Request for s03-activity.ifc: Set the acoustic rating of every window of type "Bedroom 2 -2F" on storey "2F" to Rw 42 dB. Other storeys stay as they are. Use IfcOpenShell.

First a look at what the model holds.

```python
import ifcopenshell
import ifcopenshell.util.element

model = ifcopenshell.open("s03-activity.ifc")
print(model.schema)
storey = next(s for s in model.by_type("IfcBuildingStorey") if s.Name == "2F")
windows = [e for e in ifcopenshell.util.element.get_decomposition(storey) if e.is_a("IfcWindow")]
seen = {}
for e in windows:
    element_type = ifcopenshell.util.element.get_type(e)
    key = (element_type.Name if element_type != e and element_type else None, ifcopenshell.util.element.get_pset(e, "Pset_WindowCommon", "AcousticRating"))
    seen[key] = seen.get(key, 0) + 1
for (name, value), count in sorted(seen.items(), key=str):
    print(count, "x", name, "|", value)
```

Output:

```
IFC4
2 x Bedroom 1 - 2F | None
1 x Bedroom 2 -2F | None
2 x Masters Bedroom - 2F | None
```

```python
import ifcopenshell
import ifcopenshell.api.pset
import ifcopenshell.util.element

model = ifcopenshell.open("s03-activity.ifc")

storey = next(s for s in model.by_type("IfcBuildingStorey") if s.Name == "2F")
windows = [e for e in ifcopenshell.util.element.get_decomposition(storey) if e.is_a("IfcWindow")]

count = 0
for e in windows:
    element_type = ifcopenshell.util.element.get_type(e)
    if element_type in (None, e) or element_type.Name != "Bedroom 2 -2F":
        continue
    # add_pset returns the element's existing set when there is one.
    pset = ifcopenshell.api.pset.add_pset(model, product=e, name="Pset_WindowCommon")
    ifcopenshell.api.pset.edit_pset(model, pset=pset, properties={"AcousticRating": "Rw 42 dB"})
    count += 1

print(count, "windows updated")

model.write("s03-activity_v2.ifc")
```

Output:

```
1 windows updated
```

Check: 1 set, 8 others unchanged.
